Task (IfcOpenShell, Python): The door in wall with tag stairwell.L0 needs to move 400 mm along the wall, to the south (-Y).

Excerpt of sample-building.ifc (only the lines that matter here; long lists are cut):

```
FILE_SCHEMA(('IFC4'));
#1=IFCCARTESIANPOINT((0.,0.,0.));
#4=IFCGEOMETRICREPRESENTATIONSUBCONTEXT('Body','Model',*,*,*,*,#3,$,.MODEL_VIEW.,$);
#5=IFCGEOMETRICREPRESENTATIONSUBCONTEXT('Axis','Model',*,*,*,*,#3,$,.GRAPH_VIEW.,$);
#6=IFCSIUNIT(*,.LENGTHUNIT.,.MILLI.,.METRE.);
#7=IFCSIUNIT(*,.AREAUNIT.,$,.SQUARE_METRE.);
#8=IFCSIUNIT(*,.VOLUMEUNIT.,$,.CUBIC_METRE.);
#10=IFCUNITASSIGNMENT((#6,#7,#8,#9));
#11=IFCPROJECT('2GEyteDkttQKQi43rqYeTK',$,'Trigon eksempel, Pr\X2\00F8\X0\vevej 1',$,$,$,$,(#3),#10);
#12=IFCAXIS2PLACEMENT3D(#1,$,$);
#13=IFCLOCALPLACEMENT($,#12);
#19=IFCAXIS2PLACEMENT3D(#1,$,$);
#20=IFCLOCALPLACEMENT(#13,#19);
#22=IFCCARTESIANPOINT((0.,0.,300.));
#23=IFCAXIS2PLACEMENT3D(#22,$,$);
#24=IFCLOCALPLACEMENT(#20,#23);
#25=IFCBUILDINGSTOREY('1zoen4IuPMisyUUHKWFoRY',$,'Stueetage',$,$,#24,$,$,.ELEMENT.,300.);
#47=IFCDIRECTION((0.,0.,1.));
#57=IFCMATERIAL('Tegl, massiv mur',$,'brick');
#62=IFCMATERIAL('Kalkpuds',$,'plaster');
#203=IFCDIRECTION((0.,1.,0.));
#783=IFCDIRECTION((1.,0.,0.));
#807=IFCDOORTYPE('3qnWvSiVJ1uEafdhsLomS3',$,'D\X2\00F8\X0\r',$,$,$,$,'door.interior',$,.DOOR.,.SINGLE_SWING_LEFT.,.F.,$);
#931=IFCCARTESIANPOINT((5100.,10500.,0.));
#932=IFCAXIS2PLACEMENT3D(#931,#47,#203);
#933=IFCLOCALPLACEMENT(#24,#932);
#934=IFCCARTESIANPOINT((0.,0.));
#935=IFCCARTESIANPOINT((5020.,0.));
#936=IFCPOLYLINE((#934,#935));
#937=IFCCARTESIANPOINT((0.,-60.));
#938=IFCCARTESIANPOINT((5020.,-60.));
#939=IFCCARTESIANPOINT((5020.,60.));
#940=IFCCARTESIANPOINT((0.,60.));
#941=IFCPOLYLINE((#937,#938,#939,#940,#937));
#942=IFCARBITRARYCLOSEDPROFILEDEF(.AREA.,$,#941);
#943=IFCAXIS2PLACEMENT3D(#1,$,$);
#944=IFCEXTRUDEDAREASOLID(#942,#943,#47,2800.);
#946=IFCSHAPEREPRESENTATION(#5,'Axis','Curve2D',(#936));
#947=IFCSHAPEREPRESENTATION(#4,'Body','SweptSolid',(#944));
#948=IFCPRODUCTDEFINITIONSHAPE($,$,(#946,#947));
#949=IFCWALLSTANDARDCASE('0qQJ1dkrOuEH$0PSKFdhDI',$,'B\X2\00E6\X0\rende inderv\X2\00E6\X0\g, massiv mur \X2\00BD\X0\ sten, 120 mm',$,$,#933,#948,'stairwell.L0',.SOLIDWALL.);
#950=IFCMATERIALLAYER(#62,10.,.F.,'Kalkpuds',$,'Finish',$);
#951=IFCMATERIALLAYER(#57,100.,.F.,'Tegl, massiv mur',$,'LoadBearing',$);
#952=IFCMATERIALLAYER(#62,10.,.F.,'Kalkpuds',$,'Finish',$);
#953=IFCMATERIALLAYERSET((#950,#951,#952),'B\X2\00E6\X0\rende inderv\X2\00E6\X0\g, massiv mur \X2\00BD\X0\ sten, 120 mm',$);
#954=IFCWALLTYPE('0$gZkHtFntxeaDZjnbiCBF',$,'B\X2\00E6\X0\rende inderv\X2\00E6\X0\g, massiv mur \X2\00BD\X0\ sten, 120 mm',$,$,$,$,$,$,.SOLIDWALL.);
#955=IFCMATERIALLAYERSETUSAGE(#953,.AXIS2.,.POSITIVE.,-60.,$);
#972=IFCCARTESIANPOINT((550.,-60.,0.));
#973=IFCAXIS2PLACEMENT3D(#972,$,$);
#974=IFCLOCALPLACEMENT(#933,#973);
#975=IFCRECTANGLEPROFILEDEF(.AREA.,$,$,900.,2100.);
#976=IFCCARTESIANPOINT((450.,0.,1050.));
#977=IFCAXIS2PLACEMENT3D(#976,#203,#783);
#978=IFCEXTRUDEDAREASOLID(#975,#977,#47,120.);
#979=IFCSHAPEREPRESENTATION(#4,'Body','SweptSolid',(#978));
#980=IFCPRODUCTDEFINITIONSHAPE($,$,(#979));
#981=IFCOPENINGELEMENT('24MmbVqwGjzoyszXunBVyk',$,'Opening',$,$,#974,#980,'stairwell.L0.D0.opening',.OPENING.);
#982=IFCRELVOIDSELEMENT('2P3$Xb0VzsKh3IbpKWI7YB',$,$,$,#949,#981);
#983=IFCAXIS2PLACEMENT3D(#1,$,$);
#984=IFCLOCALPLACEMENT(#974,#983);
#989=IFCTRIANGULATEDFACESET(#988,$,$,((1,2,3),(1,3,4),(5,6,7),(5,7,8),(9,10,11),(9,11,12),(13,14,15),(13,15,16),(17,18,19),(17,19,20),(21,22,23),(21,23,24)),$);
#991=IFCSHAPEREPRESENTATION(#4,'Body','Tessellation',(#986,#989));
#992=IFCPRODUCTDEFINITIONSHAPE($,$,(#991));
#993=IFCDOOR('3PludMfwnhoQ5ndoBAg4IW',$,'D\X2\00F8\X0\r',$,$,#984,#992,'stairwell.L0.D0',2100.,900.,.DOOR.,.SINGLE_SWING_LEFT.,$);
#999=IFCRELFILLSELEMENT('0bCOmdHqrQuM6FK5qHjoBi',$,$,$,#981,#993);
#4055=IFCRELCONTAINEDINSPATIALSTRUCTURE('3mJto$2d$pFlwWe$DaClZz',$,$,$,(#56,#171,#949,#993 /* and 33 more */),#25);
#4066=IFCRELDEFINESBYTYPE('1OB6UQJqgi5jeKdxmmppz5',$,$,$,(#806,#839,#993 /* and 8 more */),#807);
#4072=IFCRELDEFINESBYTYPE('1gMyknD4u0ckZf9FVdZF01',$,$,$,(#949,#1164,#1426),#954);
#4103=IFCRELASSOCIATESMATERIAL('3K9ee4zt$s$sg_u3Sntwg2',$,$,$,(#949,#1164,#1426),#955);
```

```python
import ifcopenshell
import ifcopenshell.api.geometry
import ifcopenshell.util.placement
import ifcopenshell.util.unit

model = ifcopenshell.open("sample-building.ifc")
unit_scale = ifcopenshell.util.unit.calculate_unit_scale(model)

door = model.by_id(993)
opening = door.FillsVoids[0].RelatingOpeningElement
wall = opening.VoidsElements[0].RelatingBuildingElement

wall_matrix = ifcopenshell.util.placement.get_local_placement(wall.ObjectPlacement)
shift = wall_matrix[:3, 0] * -0.4 / unit_scale
before = ifcopenshell.util.placement.get_local_placement(door.ObjectPlacement)[:3, 3].copy()

# The door is placed relative to its opening, so it follows when the opening moves.
matrix = ifcopenshell.util.placement.get_local_placement(opening.ObjectPlacement)
matrix[:3, 3] += shift
ifcopenshell.api.geometry.edit_object_placement(
    model, product=opening, matrix=matrix, is_si=False, should_transform_children=True
)

after = ifcopenshell.util.placement.get_local_placement(door.ObjectPlacement)[:3, 3]
print("door moved by", (after - before).round(3) + 0.0)

model.write("sample-building_rev.ifc")
```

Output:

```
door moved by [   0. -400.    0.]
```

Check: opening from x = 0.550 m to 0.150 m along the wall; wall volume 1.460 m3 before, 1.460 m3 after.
